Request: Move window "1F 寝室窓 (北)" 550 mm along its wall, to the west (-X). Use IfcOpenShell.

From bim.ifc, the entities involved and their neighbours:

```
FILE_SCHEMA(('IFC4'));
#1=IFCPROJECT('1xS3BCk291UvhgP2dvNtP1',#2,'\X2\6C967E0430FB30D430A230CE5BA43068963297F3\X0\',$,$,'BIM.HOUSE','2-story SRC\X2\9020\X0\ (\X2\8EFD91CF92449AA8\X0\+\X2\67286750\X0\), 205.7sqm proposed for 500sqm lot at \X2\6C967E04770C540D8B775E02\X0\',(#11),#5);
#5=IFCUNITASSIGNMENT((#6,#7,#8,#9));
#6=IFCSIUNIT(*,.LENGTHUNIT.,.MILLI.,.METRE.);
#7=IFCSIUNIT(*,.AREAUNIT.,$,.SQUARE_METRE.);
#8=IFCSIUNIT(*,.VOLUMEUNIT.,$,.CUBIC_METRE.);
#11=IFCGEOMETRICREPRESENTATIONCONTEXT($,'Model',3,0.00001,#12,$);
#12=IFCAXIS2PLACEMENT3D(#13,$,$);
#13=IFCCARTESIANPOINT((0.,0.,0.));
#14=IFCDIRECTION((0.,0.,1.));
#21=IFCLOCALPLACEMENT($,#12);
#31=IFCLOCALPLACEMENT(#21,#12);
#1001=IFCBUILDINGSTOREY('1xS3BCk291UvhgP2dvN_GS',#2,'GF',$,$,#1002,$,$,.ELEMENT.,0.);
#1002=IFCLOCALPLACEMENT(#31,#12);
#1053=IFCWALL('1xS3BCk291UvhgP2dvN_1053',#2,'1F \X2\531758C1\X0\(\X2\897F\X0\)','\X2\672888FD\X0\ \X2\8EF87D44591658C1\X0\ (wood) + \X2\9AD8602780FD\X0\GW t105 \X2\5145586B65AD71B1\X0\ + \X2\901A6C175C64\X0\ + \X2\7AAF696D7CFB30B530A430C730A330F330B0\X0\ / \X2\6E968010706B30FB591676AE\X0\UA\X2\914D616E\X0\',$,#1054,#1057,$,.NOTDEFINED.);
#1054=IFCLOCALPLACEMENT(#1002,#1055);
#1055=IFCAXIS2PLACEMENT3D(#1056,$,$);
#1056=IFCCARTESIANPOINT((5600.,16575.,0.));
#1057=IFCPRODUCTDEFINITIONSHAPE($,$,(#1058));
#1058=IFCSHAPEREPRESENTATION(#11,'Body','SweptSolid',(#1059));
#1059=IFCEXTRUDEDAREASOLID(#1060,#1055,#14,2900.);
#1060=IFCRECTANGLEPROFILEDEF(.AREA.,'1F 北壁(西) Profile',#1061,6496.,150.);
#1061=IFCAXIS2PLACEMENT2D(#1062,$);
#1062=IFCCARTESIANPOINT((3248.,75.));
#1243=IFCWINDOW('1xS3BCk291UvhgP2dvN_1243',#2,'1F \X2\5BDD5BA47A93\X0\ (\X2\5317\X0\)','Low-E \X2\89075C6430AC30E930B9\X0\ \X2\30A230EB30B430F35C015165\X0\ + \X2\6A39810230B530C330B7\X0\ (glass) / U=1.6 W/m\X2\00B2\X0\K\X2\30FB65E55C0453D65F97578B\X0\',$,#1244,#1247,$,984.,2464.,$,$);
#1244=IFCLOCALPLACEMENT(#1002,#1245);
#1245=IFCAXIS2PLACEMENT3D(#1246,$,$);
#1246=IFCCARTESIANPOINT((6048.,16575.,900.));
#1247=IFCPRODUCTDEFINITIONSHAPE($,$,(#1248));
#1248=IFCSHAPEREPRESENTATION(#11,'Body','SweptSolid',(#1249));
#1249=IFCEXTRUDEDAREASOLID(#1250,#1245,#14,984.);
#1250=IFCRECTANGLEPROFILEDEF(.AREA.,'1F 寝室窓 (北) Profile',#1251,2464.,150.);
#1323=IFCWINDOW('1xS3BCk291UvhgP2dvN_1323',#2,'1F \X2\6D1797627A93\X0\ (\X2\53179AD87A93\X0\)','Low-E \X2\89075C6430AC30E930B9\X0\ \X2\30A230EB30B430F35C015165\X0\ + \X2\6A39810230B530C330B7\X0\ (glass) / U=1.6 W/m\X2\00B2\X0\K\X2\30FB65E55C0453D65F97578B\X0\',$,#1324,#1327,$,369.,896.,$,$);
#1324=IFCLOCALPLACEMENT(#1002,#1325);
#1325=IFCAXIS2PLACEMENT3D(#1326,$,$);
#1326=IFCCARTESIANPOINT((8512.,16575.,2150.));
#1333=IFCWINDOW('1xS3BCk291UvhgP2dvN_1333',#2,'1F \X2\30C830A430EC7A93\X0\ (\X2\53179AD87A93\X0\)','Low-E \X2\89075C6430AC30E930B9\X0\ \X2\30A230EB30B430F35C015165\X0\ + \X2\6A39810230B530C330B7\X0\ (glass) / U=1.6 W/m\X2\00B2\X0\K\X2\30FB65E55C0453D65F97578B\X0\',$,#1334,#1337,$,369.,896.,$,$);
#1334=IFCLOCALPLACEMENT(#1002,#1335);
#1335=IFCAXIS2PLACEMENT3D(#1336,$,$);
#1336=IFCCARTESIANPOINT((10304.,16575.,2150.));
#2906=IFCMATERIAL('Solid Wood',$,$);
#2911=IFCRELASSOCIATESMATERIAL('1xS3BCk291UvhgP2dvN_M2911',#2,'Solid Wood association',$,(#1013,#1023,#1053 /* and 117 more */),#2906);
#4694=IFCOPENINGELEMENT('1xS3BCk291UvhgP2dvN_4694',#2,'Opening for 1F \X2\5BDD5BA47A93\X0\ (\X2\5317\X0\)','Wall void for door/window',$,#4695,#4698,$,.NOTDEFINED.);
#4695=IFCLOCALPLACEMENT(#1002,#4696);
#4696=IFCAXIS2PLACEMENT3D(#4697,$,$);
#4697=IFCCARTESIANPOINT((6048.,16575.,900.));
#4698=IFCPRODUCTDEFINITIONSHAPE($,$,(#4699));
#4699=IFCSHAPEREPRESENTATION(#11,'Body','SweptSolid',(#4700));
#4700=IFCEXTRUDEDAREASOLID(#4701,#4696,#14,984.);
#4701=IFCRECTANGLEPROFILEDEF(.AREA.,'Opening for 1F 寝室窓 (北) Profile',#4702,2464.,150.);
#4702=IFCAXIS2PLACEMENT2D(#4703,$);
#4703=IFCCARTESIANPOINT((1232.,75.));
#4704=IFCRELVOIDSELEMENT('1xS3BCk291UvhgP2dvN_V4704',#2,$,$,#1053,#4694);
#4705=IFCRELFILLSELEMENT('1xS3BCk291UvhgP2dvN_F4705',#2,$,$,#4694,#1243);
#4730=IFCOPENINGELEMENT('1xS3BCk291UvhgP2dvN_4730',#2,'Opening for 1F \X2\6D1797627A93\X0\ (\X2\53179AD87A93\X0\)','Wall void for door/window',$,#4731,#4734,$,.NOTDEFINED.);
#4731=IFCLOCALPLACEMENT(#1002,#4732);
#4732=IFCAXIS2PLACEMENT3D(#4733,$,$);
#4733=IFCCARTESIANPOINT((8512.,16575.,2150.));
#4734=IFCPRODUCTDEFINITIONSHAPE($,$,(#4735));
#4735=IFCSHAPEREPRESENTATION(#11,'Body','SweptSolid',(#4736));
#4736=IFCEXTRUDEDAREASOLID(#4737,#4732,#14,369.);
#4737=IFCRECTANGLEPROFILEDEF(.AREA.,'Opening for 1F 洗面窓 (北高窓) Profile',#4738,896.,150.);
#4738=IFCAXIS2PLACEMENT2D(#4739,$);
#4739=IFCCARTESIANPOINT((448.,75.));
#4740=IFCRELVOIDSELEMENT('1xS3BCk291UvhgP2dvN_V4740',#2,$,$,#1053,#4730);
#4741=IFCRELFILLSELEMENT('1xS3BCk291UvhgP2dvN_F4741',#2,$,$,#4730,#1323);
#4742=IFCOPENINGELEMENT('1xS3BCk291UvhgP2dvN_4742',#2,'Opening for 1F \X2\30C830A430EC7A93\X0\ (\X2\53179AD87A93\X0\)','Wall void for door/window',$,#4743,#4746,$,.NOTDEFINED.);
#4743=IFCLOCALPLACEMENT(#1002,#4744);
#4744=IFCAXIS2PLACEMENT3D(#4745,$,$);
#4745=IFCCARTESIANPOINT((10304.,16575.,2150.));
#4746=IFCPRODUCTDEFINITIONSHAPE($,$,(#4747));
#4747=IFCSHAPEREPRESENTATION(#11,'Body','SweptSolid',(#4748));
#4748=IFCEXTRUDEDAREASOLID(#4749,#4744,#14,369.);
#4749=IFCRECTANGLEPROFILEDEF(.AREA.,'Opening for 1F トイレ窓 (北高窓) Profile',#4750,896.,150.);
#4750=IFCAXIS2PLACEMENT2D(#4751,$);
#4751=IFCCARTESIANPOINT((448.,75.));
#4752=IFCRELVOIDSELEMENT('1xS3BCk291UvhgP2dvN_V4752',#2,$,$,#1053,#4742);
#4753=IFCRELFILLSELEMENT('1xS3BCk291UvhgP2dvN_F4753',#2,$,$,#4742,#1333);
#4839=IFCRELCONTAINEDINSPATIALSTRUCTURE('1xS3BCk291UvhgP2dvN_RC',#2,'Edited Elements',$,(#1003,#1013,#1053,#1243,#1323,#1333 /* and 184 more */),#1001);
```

```python
import ifcopenshell
import ifcopenshell.api.geometry
import ifcopenshell.util.placement
import ifcopenshell.util.unit

model = ifcopenshell.open("bim.ifc")
unit_scale = ifcopenshell.util.unit.calculate_unit_scale(model)

window = model.by_guid("1xS3BCk291UvhgP2dvN_1243")
opening = window.FillsVoids[0].RelatingOpeningElement
wall = opening.VoidsElements[0].RelatingBuildingElement

wall_matrix = ifcopenshell.util.placement.get_local_placement(wall.ObjectPlacement)
shift = wall_matrix[:3, 0] * -0.55 / unit_scale
before = ifcopenshell.util.placement.get_local_placement(window.ObjectPlacement)[:3, 3].copy()

# The window is not placed relative to its opening, so move both.
for product in (opening, window):
    matrix = ifcopenshell.util.placement.get_local_placement(product.ObjectPlacement)
    matrix[:3, 3] += shift
    ifcopenshell.api.geometry.edit_object_placement(model, product=product, matrix=matrix, is_si=False)

after = ifcopenshell.util.placement.get_local_placement(window.ObjectPlacement)[:3, 3]
print("window moved by", (after - before).round(3) + 0.0)

model.write("bim-out.ifc")
```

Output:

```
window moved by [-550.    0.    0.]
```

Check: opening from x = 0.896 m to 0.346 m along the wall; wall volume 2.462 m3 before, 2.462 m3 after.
